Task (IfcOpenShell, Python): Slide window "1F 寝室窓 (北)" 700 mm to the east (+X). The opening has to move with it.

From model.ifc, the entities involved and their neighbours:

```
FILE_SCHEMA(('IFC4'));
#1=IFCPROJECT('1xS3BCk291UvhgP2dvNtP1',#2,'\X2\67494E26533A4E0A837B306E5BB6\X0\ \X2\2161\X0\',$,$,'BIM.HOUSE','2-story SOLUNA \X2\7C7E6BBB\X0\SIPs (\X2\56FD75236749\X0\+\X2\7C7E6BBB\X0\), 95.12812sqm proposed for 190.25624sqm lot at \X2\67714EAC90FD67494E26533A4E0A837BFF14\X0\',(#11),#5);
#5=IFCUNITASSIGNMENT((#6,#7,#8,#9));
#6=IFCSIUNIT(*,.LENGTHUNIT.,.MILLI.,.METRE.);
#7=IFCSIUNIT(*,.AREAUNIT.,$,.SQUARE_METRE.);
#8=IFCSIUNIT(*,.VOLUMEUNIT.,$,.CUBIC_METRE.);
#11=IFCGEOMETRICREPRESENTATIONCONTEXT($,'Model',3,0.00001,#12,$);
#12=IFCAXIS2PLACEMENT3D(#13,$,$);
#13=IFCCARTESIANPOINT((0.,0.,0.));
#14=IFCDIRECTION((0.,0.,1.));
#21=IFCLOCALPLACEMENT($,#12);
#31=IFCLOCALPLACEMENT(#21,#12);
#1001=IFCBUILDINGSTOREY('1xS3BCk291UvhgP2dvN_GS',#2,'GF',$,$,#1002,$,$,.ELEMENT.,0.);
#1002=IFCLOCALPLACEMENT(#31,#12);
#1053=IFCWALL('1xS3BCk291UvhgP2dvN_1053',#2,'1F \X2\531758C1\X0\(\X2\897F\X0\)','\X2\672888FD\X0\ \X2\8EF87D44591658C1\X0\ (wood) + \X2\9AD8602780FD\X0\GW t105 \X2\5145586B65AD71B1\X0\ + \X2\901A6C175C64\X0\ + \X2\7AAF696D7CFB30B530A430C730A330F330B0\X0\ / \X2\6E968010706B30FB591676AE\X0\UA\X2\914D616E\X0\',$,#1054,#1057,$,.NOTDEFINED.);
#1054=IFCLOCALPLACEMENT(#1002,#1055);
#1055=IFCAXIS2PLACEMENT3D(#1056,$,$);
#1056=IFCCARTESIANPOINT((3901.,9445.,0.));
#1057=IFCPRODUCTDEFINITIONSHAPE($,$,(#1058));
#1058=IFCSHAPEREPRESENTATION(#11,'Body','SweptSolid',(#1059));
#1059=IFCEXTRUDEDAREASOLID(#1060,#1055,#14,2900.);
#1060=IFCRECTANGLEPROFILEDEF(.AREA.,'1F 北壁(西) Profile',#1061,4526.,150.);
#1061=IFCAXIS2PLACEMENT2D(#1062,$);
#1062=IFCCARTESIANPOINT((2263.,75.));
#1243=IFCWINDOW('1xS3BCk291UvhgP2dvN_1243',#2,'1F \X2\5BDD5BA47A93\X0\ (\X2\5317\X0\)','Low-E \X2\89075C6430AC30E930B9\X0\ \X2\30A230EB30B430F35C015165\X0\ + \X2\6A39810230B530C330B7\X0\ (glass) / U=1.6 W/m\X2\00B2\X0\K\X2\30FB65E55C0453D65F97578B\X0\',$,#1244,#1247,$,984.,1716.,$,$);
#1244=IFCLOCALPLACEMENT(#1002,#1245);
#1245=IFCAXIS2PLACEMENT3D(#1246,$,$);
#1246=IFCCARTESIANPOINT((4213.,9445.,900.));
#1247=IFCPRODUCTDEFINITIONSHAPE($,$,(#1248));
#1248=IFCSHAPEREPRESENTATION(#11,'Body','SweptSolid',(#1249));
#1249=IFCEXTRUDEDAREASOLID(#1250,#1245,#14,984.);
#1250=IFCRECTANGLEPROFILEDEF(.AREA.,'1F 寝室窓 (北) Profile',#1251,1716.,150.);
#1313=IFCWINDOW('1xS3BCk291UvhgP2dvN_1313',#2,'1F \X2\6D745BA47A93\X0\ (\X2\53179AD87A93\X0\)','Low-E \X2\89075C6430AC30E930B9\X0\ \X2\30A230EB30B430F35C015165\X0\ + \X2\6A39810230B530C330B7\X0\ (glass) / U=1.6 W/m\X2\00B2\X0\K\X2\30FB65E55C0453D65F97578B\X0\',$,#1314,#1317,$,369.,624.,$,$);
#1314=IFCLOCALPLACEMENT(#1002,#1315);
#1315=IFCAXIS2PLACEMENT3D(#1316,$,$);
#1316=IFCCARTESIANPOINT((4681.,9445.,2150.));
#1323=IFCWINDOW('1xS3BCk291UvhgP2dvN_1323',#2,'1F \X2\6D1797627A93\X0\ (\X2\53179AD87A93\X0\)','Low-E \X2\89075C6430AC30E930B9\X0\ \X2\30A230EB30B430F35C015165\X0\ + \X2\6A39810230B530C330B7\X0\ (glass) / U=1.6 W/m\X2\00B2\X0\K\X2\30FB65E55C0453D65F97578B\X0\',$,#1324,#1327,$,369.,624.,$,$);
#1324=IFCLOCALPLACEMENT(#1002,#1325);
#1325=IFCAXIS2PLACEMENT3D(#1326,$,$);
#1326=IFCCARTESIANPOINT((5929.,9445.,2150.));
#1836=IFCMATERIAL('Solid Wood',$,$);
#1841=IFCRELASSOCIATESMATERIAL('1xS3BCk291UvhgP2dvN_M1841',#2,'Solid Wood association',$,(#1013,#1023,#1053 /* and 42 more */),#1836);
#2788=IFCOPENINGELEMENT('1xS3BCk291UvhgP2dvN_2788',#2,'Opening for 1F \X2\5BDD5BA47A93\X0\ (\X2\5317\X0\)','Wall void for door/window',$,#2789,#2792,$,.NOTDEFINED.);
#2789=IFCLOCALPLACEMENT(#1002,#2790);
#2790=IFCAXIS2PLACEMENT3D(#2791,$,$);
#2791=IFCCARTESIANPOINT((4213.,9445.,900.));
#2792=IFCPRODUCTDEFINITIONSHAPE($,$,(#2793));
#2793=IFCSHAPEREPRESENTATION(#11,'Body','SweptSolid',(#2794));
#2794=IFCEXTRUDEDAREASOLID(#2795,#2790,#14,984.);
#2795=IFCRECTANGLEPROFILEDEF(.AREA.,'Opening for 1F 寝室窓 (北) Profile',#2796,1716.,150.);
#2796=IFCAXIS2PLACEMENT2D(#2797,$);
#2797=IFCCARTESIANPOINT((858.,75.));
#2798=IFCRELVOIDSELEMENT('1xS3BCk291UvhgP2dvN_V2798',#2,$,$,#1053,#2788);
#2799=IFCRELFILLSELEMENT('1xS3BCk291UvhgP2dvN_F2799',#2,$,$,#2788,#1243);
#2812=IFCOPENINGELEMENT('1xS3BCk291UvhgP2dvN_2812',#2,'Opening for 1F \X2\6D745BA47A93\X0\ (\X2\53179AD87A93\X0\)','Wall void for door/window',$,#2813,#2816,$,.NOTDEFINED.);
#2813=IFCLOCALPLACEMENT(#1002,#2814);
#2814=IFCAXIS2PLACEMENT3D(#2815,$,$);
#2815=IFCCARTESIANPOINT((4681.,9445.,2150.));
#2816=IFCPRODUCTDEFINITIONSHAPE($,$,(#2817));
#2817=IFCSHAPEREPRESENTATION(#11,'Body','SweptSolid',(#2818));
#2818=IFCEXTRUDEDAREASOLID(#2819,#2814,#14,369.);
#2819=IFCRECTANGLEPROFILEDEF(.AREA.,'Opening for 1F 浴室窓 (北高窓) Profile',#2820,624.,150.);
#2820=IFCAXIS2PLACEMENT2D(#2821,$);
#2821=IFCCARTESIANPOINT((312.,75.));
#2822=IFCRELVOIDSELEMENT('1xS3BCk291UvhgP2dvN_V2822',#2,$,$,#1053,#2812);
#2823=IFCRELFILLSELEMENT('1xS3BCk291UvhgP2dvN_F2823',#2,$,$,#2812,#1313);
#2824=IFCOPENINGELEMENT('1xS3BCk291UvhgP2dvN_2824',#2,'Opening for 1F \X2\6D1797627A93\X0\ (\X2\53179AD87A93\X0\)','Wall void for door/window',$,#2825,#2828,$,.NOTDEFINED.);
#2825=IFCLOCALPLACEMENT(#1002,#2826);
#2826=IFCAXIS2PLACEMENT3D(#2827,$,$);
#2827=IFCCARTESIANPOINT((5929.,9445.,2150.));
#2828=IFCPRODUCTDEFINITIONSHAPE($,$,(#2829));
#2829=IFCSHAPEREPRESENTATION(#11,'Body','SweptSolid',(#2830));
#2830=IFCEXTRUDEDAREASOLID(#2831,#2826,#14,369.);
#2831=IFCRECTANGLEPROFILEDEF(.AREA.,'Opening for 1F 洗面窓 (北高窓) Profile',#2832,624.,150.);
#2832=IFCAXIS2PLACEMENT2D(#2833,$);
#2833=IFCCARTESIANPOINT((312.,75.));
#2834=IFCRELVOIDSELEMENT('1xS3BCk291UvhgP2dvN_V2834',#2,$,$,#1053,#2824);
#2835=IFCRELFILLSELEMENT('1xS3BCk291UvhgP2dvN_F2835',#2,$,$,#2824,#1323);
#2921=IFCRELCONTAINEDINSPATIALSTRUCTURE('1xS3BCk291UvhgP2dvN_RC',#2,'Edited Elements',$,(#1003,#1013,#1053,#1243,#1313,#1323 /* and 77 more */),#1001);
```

```python
import ifcopenshell
import ifcopenshell.api.geometry
import ifcopenshell.util.placement
import ifcopenshell.util.unit

model = ifcopenshell.open("model.ifc")
unit_scale = ifcopenshell.util.unit.calculate_unit_scale(model)

window = model.by_id(1243)
opening = window.FillsVoids[0].RelatingOpeningElement
wall = opening.VoidsElements[0].RelatingBuildingElement

wall_matrix = ifcopenshell.util.placement.get_local_placement(wall.ObjectPlacement)
shift = wall_matrix[:3, 0] * 0.7 / unit_scale
before = ifcopenshell.util.placement.get_local_placement(window.ObjectPlacement)[:3, 3].copy()

# The window is not placed relative to its opening, so move both.
for product in (opening, window):
    matrix = ifcopenshell.util.placement.get_local_placement(product.ObjectPlacement)
    matrix[:3, 3] += shift
    ifcopenshell.api.geometry.edit_object_placement(model, product=product, matrix=matrix, is_si=False)

after = ifcopenshell.util.placement.get_local_placement(window.ObjectPlacement)[:3, 3]
print("window moved by", (after - before).round(3) + 0.0)

model.write("model-out.ifc")
```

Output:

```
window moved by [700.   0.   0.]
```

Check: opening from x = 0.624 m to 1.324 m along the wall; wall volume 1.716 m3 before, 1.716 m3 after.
